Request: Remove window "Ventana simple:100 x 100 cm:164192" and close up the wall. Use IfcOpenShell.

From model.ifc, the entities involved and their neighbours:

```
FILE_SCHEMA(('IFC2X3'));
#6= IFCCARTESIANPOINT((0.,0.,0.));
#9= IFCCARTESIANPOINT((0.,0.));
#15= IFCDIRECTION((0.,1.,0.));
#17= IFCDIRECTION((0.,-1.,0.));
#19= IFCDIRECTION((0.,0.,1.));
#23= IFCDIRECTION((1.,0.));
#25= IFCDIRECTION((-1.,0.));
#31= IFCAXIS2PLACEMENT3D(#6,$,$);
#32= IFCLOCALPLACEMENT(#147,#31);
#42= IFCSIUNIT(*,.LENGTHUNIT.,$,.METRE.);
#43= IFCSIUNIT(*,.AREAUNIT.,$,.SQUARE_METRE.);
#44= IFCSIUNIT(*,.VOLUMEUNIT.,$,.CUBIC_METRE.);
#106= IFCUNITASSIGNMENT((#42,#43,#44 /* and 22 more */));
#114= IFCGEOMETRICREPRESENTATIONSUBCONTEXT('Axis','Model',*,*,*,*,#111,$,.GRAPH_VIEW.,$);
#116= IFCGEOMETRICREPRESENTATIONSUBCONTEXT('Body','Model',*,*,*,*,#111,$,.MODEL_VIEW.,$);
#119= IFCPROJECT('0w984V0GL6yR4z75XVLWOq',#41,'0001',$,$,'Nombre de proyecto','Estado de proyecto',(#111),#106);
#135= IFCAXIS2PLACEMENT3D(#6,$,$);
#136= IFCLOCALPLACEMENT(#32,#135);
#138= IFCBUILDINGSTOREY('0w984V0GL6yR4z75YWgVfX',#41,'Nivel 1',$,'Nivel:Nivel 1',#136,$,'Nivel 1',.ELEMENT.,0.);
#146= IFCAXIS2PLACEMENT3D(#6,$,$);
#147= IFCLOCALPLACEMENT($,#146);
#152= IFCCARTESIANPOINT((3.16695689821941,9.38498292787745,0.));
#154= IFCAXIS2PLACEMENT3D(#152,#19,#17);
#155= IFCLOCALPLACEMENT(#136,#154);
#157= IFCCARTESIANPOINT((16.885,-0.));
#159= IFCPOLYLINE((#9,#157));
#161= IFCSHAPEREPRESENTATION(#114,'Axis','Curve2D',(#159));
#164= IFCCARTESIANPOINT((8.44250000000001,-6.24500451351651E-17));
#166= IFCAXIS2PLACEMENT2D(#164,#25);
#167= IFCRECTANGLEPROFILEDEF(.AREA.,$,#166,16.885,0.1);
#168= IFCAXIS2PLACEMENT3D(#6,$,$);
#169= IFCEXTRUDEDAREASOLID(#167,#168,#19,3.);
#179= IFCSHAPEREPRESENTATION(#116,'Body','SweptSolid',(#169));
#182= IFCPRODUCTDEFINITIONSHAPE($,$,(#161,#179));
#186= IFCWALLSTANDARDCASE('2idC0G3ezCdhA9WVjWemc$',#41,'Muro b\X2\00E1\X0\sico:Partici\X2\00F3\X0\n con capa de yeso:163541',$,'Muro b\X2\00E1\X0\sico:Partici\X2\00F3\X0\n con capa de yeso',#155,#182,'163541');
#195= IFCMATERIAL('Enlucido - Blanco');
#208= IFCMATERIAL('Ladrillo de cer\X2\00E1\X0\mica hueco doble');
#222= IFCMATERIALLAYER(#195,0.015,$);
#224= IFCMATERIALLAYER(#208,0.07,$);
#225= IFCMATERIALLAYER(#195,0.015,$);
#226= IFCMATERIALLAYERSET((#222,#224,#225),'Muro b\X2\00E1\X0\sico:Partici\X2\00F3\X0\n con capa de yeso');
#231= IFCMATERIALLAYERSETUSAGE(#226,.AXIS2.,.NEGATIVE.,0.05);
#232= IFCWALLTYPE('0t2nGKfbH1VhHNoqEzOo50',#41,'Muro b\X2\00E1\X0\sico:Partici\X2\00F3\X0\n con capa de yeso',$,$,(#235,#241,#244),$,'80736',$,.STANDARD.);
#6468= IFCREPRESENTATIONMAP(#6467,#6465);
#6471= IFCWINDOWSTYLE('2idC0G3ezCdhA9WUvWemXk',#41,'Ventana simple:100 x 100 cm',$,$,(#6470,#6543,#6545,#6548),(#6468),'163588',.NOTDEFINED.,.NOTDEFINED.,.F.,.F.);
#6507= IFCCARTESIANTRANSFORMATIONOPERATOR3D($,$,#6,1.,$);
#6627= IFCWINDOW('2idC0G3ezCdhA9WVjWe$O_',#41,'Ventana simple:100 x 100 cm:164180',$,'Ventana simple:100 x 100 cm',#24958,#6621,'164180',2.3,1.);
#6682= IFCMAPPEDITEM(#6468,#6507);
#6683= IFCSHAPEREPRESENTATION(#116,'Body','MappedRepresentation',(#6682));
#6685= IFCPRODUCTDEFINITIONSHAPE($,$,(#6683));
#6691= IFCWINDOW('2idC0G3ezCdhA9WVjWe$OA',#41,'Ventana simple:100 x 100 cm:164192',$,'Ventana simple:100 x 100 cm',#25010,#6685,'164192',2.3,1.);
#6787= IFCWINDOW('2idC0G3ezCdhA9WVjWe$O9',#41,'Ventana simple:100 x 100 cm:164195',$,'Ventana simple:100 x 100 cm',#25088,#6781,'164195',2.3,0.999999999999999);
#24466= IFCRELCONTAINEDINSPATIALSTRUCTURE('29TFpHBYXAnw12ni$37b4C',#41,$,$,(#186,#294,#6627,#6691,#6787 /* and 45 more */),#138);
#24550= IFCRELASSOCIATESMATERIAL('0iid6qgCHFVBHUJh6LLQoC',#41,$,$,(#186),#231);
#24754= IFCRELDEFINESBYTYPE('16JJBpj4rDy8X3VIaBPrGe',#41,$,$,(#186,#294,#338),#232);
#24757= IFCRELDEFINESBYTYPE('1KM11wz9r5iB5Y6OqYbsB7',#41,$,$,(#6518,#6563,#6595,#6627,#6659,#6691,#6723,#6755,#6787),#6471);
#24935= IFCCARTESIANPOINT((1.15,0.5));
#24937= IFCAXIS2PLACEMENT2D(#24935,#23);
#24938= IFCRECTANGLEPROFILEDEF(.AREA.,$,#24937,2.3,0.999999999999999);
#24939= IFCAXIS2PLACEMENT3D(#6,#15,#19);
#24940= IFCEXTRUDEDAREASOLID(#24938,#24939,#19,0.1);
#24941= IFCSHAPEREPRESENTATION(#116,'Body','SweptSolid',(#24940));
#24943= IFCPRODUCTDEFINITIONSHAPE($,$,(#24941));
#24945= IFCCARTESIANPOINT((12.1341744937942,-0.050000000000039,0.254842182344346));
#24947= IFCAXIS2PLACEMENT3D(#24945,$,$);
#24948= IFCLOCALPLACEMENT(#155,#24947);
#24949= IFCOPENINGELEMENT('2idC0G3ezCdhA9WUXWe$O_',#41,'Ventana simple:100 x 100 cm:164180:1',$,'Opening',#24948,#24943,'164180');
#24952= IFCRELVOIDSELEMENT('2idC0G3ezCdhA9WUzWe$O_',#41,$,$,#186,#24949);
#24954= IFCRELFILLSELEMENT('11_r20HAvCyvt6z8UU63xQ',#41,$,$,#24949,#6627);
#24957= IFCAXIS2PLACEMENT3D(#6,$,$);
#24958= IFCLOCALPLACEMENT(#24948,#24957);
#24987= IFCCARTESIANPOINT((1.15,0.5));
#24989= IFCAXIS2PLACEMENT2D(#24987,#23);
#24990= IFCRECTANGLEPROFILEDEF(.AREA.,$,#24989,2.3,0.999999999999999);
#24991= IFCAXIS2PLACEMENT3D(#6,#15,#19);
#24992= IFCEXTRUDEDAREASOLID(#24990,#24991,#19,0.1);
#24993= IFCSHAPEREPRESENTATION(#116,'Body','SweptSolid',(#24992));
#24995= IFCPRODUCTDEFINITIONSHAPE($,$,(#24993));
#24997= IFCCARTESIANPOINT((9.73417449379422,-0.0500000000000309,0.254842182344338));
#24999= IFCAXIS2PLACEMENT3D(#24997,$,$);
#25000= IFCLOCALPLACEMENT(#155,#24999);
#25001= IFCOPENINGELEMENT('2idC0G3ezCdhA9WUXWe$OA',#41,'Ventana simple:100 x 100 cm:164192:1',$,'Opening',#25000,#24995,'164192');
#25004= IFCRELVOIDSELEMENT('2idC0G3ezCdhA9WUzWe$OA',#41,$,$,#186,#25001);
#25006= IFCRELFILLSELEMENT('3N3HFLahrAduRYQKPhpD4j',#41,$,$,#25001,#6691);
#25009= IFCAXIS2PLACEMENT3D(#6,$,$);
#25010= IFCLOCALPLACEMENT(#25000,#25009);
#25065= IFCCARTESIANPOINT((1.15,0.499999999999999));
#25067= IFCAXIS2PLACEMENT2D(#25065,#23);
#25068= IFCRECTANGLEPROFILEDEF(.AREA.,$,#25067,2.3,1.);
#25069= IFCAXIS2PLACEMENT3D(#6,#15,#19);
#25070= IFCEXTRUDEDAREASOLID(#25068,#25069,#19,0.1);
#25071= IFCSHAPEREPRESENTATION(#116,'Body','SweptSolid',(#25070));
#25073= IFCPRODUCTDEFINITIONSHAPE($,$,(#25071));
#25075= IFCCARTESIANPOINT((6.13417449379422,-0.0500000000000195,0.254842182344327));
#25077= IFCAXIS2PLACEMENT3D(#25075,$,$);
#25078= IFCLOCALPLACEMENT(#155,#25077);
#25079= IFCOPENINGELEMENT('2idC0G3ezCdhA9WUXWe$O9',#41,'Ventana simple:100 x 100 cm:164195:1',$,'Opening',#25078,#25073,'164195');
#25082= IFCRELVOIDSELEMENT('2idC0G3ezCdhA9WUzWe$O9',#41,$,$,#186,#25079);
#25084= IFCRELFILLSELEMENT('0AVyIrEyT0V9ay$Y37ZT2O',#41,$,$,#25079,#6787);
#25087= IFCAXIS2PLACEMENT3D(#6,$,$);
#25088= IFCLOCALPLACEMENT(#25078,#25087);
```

```python
import ifcopenshell
import ifcopenshell.api.feature
import ifcopenshell.api.root
import ifcopenshell.geom
import ifcopenshell.util.shape

model = ifcopenshell.open("model.ifc")
settings = ifcopenshell.geom.settings()


def volume(element):
    """Net volume in cubic metres, openings subtracted."""
    shape = ifcopenshell.geom.create_shape(settings, element)
    return ifcopenshell.util.shape.get_volume(shape.geometry)


window = model.by_id(6691)
opening = window.FillsVoids[0].RelatingOpeningElement
wall = opening.VoidsElements[0].RelatingBuildingElement
before = volume(wall)

ifcopenshell.api.root.remove_product(model, product=window)
ifcopenshell.api.feature.remove_feature(model, feature=opening)

after = volume(wall)

print(f"wall volume {before:.3f} -> {after:.3f} m3")

model.write("model-out.ifc")
```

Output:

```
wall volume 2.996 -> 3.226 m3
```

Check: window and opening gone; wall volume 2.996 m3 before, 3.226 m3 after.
